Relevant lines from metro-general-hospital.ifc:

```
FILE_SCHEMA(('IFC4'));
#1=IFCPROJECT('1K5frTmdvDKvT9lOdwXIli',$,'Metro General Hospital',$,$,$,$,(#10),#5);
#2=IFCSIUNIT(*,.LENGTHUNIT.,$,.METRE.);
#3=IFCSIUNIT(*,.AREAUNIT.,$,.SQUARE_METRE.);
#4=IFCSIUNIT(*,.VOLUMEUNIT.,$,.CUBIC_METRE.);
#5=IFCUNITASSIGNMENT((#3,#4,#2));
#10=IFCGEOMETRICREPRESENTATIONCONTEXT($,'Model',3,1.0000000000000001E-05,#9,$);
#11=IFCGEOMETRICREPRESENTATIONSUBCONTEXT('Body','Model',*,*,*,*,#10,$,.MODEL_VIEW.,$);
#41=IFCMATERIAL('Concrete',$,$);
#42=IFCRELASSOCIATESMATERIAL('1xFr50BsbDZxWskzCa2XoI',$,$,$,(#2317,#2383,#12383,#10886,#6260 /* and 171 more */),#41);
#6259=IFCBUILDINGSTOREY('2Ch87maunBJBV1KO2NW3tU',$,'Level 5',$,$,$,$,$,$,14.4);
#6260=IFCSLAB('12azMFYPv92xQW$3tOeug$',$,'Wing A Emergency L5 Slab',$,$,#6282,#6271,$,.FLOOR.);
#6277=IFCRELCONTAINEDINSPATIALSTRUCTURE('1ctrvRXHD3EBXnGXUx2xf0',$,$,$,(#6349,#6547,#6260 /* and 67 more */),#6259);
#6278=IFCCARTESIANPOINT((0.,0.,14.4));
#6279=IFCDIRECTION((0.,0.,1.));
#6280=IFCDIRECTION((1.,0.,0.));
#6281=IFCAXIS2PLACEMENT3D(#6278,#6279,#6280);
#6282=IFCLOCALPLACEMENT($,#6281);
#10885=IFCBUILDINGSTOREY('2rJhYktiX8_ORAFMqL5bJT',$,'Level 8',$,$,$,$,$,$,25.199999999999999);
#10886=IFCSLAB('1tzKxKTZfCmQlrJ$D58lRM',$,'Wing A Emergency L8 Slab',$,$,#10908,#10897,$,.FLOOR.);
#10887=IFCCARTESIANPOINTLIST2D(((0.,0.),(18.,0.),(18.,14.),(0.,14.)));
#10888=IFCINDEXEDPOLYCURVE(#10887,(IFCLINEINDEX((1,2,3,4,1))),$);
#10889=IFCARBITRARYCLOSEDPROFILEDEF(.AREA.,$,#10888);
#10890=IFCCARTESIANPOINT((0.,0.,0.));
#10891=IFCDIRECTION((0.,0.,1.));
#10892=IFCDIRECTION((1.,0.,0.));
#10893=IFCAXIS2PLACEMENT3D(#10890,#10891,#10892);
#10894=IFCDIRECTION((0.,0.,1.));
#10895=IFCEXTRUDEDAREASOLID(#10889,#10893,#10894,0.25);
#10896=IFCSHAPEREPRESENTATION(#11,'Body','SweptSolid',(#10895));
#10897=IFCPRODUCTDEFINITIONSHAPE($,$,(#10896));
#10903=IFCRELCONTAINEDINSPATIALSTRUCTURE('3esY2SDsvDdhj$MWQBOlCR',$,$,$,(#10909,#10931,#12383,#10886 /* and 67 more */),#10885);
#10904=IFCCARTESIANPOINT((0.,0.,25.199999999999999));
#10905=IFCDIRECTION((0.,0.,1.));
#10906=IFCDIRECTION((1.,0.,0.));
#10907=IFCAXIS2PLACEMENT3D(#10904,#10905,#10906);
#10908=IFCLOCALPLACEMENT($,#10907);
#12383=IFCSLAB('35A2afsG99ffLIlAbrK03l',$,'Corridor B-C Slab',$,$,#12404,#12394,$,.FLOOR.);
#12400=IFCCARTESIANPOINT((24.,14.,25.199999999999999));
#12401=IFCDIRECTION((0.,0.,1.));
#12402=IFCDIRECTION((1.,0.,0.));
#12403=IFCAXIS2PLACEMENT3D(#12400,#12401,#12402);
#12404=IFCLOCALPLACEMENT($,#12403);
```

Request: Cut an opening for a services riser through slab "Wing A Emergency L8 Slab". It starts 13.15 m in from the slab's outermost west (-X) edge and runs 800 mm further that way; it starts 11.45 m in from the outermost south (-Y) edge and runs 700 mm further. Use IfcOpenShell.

```python
import numpy as np
import ifcopenshell
import ifcopenshell.api.feature
import ifcopenshell.api.geometry
import ifcopenshell.api.root
import ifcopenshell.geom
import ifcopenshell.util.placement
import ifcopenshell.util.representation
import ifcopenshell.util.shape
import ifcopenshell.util.unit

model = ifcopenshell.open("metro-general-hospital.ifc")
unit_scale = ifcopenshell.util.unit.calculate_unit_scale(model)
settings = ifcopenshell.geom.settings()


def volume(element):
    """Net volume in cubic metres, openings subtracted."""
    shape = ifcopenshell.geom.create_shape(settings, element)
    return ifcopenshell.util.shape.get_volume(shape.geometry)


slab = model.by_guid("1tzKxKTZfCmQlrJ$D58lRM")
before = volume(slab)

# Extent in the slab's own axes, in metres. The edges named are its -X and -Y sides.
slab_shape = ifcopenshell.geom.create_shape(settings, slab)
vertices = ifcopenshell.util.shape.get_vertices(slab_shape.geometry)
x_min, y_min, bottom = vertices.min(axis=0)
top = vertices[:, 2].max()

opening = ifcopenshell.api.root.create_entity(model, ifc_class="IfcOpeningElement", name="Services riser opening", predefined_type="OPENING")
context = ifcopenshell.util.representation.get_context(model, "Model", "Body", "MODEL_VIEW")
width, depth = 0.8, 0.7
outline = [(0.0, 0.0), (width, 0.0), (width, depth), (0.0, depth), (0.0, 0.0)]
# Overshoot both faces by 50 mm so the cut is clean.
shape = ifcopenshell.api.geometry.add_slab_representation(
    model, context=context, depth=top - bottom + 0.1, polyline=outline
)
ifcopenshell.api.geometry.assign_representation(model, product=opening, representation=shape)

matrix = ifcopenshell.util.placement.get_local_placement(slab.ObjectPlacement)
matrix[:, 3] = matrix @ np.append(np.array([x_min + 13.15, y_min + 11.45, bottom - 0.05]) / unit_scale, 1.0)
ifcopenshell.api.geometry.edit_object_placement(model, product=opening, matrix=matrix, is_si=False)
ifcopenshell.api.feature.add_feature(model, feature=opening, element=slab)

after = volume(slab)

print(f"slab volume {before:.3f} -> {after:.3f} m3")

model.write("metro-general-hospital-out.ifc")
```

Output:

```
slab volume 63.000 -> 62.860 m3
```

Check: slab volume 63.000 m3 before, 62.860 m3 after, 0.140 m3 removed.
